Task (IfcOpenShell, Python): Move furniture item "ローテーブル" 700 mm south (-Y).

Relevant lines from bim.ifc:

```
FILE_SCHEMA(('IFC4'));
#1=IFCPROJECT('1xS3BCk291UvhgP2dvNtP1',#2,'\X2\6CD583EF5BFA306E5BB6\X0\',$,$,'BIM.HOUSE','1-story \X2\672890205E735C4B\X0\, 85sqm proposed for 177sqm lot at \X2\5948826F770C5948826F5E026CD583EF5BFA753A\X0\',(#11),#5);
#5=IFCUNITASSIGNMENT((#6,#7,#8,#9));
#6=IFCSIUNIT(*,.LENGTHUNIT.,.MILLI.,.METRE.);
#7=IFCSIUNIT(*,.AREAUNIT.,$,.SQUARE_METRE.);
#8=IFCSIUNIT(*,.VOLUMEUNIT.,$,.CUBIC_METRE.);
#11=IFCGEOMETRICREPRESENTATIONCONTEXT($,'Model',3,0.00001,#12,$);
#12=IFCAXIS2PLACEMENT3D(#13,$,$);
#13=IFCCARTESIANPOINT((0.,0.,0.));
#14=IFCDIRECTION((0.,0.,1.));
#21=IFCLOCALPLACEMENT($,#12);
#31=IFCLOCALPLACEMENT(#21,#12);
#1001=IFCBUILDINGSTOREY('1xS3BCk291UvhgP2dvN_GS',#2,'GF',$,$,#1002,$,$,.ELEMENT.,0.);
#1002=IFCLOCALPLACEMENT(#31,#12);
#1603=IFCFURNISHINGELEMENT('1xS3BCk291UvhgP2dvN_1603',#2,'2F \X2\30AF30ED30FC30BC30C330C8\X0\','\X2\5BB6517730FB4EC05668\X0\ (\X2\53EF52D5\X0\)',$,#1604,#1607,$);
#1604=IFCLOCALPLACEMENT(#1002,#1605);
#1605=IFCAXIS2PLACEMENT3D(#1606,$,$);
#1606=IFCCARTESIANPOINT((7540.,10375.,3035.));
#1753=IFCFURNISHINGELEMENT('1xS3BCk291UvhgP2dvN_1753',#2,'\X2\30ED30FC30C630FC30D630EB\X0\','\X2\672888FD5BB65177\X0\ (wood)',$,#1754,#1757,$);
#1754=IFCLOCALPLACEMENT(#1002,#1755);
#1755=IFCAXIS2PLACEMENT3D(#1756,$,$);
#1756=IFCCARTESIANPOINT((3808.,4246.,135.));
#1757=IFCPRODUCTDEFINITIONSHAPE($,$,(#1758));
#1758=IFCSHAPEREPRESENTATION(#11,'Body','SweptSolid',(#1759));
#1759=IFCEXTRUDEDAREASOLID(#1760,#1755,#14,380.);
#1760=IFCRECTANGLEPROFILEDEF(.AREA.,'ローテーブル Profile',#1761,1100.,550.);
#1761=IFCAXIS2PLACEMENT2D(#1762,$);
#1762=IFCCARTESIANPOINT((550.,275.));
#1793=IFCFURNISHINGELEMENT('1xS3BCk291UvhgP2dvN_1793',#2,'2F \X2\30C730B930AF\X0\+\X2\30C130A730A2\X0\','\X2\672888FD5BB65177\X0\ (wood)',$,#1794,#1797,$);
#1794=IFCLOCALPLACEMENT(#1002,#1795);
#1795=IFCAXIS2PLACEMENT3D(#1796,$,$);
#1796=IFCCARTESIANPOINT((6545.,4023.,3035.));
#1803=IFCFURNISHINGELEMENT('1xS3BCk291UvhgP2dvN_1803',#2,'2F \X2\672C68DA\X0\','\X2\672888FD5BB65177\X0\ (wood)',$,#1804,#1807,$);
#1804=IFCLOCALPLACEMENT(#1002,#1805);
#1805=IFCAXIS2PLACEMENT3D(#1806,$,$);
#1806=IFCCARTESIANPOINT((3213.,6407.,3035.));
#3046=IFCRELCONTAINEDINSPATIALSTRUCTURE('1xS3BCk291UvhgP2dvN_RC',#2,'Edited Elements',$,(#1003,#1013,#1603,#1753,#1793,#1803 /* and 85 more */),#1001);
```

```python
import ifcopenshell
import ifcopenshell.api.geometry
import ifcopenshell.util.placement
import ifcopenshell.util.unit

model = ifcopenshell.open("bim.ifc")
unit_scale = ifcopenshell.util.unit.calculate_unit_scale(model)

item = model.by_guid("1xS3BCk291UvhgP2dvN_1753")
matrix = ifcopenshell.util.placement.get_local_placement(item.ObjectPlacement)
matrix[1, 3] -= 0.7 / unit_scale
ifcopenshell.api.geometry.edit_object_placement(model, product=item, matrix=matrix, is_si=False)

print(ifcopenshell.util.placement.get_local_placement(item.ObjectPlacement).round(3) + 0.0)

model.write("bim-out.ifc")
```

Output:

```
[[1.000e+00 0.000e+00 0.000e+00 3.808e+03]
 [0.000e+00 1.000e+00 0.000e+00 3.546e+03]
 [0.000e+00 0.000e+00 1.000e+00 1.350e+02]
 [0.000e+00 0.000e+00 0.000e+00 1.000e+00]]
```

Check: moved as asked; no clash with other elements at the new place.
